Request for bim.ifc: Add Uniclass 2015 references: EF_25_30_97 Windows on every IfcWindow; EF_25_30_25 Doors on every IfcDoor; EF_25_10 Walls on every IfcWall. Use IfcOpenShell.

First a look at what the model holds.

```python
import ifcopenshell

model = ifcopenshell.open("bim.ifc")
print(model.schema)
print("classifications:", [c.Name for c in model.by_type("IfcClassification")])
for ifc_class in ("IfcDoor", "IfcRoof", "IfcStair", "IfcWall", "IfcWindow"):
    print(ifc_class, len(model.by_type(ifc_class)))
```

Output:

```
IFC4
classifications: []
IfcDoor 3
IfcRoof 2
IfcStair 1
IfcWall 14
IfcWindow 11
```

```python
import ifcopenshell
import ifcopenshell.api.classification

model = ifcopenshell.open("bim.ifc")

system = ifcopenshell.api.classification.add_classification(model, classification="Uniclass 2015")

codes = {
    "IfcWindow": ("EF_25_30_97", "Windows"),
    "IfcDoor": ("EF_25_30_25", "Doors"),
    "IfcWall": ("EF_25_10", "Walls"),
}
for ifc_class, (code, name) in codes.items():
    products = model.by_type(ifc_class)
    ifcopenshell.api.classification.add_reference(
        model, products=products, classification=system, identification=code, name=name
    )
    print(code, len(products))

model.write("bim_updated.ifc")
```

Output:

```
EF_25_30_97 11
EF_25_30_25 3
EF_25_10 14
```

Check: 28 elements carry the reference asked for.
